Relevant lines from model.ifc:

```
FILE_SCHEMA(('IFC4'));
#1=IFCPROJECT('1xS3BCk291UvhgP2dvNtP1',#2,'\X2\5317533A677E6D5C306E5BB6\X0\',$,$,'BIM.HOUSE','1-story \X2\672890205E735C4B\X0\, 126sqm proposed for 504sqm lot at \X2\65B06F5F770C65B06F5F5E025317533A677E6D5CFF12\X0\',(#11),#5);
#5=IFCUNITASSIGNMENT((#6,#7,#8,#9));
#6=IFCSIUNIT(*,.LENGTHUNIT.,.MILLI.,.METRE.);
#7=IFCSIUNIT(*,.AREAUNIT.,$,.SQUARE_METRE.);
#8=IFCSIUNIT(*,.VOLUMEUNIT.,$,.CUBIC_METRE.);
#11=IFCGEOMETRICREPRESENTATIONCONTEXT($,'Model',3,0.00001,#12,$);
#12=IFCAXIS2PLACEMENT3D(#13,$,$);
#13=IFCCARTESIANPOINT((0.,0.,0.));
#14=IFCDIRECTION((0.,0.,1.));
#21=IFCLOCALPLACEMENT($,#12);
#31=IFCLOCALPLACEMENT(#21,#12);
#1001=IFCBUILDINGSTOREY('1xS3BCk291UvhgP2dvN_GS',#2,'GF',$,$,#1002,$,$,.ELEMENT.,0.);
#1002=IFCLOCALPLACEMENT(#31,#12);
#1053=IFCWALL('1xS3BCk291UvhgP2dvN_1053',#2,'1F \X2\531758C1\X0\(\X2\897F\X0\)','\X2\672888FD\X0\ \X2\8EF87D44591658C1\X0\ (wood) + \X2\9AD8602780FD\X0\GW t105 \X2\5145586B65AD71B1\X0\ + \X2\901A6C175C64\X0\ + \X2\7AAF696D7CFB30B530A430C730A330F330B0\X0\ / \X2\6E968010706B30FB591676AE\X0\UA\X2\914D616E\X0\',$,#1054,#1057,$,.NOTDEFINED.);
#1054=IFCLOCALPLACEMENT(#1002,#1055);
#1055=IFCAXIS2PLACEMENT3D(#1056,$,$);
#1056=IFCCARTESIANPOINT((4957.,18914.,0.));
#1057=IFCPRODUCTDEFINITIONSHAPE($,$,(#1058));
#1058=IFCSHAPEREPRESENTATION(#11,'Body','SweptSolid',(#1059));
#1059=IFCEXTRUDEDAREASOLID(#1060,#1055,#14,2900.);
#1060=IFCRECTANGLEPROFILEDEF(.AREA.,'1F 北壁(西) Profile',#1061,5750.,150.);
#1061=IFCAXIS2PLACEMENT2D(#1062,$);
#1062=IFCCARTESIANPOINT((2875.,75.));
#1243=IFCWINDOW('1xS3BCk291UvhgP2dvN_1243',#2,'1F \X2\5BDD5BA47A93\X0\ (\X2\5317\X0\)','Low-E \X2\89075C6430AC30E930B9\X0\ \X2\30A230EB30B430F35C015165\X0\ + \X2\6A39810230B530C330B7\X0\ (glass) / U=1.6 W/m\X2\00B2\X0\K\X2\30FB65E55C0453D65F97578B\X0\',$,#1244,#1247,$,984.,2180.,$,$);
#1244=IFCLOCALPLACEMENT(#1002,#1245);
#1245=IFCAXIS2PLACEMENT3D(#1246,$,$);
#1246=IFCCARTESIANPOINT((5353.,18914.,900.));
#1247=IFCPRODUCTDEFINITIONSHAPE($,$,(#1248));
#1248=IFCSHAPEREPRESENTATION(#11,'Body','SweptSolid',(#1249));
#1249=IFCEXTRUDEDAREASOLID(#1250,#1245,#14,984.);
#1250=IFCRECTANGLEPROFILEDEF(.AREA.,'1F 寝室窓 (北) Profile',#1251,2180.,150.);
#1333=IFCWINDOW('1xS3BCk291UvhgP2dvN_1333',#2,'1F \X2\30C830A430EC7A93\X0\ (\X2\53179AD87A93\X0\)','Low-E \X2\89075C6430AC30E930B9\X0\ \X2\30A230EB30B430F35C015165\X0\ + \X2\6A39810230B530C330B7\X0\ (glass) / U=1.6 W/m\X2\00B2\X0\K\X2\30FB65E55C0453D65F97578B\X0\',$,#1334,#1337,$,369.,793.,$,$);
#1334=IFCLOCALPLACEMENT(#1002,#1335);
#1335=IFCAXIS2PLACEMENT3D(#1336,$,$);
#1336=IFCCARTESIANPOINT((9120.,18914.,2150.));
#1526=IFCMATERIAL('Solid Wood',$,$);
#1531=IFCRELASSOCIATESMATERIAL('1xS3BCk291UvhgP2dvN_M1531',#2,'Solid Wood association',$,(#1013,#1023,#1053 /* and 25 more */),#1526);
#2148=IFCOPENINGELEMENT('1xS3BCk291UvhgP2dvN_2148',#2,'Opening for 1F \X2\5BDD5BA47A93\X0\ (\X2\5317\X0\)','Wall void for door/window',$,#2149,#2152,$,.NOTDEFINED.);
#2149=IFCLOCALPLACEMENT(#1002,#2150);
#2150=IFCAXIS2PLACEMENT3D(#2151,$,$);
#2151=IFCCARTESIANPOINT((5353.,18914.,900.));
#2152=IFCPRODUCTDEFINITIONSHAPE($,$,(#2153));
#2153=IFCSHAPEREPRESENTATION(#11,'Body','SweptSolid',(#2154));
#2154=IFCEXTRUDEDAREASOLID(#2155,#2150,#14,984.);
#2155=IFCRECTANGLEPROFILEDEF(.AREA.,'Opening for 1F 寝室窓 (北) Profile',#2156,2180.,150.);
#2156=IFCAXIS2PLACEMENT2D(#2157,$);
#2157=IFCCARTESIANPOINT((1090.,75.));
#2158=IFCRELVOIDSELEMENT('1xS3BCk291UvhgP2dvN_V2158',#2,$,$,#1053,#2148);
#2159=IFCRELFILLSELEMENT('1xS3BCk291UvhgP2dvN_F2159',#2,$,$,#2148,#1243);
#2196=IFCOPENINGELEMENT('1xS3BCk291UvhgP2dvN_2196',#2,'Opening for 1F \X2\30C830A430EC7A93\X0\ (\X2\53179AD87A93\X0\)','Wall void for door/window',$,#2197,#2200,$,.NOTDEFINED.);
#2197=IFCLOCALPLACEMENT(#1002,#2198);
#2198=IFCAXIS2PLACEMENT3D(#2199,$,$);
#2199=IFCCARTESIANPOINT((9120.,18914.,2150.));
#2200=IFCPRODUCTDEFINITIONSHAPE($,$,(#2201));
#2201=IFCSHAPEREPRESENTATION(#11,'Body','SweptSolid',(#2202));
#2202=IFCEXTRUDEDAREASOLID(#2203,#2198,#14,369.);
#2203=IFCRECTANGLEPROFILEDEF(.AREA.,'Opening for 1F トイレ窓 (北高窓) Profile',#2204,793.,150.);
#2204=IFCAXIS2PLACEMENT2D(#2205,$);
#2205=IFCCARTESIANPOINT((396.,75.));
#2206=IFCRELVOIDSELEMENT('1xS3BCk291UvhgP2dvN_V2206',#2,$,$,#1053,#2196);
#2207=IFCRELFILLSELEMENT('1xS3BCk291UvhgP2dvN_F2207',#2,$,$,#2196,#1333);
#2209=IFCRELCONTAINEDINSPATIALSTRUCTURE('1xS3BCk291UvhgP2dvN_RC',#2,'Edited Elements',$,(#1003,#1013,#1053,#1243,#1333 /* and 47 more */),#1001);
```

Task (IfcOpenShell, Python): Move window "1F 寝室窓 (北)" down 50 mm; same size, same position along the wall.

```python
import numpy as np
import ifcopenshell
import ifcopenshell.api.geometry
import ifcopenshell.util.placement
import ifcopenshell.util.unit

model = ifcopenshell.open("model.ifc")
unit_scale = ifcopenshell.util.unit.calculate_unit_scale(model)

window = model.by_guid("1xS3BCk291UvhgP2dvN_1243")
opening = window.FillsVoids[0].RelatingOpeningElement
dz = -0.05 / unit_scale

shift = np.array([0.0, 0.0, dz])
# The window is not placed relative to its opening, so move both.
for product in (opening, window):
    matrix = ifcopenshell.util.placement.get_local_placement(product.ObjectPlacement)
    matrix[:3, 3] += shift
    ifcopenshell.api.geometry.edit_object_placement(model, product=product, matrix=matrix, is_si=False)

print(f"moved by {dz * unit_scale:+.3f} m")

model.write("model_edited.ifc")
```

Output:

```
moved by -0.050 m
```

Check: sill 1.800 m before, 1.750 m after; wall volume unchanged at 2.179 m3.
